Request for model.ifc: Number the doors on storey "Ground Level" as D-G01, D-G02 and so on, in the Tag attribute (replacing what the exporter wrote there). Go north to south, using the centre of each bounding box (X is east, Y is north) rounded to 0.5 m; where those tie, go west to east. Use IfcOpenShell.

First a look at what the model holds.

```python
import ifcopenshell
import ifcopenshell.util.element
import ifcopenshell.util.placement

model = ifcopenshell.open("model.ifc")
print(model.schema)
storey = next(s for s in model.by_type("IfcBuildingStorey") if s.Name == "Ground Level")
doors = [e for e in ifcopenshell.util.element.get_decomposition(storey) if e.is_a("IfcDoor")]
for e in sorted(doors, key=lambda e: e.id()):
    origin = ifcopenshell.util.placement.get_local_placement(e.ObjectPlacement)[:3, 3]
    print(e.id(), e.Tag, e.Name, origin.round(2) + 0.0, sep=" | ")
```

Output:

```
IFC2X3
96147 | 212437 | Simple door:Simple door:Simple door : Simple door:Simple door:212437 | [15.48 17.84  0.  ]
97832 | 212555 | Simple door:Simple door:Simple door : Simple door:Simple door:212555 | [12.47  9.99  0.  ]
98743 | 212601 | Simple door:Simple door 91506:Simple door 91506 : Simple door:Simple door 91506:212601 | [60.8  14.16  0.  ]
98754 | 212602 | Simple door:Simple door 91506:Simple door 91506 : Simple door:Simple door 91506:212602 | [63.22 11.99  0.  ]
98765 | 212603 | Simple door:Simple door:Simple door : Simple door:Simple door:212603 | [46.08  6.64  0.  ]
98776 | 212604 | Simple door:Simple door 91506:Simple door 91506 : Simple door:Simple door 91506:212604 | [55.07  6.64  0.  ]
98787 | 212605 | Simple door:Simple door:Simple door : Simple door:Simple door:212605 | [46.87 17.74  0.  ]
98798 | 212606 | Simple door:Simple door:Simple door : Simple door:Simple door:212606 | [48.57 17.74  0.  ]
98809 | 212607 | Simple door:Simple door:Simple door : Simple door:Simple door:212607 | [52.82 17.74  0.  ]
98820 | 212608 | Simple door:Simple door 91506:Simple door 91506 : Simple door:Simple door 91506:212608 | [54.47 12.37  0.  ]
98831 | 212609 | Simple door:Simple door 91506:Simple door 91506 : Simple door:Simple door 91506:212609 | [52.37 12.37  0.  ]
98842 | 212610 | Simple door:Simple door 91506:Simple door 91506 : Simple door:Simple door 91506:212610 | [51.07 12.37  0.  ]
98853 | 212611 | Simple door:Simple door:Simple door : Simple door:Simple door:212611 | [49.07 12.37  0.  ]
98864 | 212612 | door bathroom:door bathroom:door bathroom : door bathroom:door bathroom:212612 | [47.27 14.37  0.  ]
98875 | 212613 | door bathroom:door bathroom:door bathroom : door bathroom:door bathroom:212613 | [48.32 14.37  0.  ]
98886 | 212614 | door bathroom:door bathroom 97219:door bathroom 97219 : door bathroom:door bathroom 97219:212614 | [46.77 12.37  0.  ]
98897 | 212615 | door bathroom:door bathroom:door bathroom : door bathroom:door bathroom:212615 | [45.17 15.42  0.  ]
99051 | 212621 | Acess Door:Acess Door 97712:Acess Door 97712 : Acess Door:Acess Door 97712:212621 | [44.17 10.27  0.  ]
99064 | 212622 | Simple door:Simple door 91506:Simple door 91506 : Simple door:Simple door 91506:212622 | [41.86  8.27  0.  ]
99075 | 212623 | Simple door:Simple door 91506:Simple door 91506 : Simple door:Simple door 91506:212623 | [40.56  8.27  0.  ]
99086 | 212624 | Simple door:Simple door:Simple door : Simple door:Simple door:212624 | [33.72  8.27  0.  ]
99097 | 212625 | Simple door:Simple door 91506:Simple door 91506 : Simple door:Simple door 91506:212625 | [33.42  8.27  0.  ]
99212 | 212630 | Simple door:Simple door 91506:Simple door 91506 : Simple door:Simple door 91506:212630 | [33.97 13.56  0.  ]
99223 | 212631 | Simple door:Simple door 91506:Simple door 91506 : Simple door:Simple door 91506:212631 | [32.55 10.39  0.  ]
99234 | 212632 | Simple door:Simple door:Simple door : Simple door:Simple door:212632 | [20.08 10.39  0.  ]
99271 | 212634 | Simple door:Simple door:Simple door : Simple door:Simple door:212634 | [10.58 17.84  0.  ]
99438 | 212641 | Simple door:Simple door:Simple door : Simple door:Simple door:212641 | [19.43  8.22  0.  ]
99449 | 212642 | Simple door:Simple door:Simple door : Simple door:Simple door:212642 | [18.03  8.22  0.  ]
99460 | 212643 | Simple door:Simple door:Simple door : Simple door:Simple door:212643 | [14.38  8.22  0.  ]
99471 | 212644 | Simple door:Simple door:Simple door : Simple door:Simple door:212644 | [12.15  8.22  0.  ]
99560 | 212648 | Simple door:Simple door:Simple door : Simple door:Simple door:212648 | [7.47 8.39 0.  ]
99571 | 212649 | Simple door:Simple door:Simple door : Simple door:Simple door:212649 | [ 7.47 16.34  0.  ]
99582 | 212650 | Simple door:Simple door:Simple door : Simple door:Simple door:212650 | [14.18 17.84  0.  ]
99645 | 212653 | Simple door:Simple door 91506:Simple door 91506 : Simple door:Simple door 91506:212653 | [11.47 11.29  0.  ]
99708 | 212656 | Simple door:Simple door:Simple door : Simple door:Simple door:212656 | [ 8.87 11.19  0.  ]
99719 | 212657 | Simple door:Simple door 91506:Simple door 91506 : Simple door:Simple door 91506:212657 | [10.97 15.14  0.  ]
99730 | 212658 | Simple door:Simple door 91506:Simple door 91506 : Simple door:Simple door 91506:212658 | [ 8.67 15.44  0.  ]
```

```python
import ifcopenshell
import ifcopenshell.geom
import ifcopenshell.util.element
import ifcopenshell.util.shape

model = ifcopenshell.open("model.ifc")
settings = ifcopenshell.geom.settings()
settings.set("use-world-coords", True)


def centre(element):
    shape = ifcopenshell.geom.create_shape(settings, element)
    return ifcopenshell.util.shape.get_bbox_centroid(shape.geometry)


storey = next(s for s in model.by_type("IfcBuildingStorey") if s.Name == "Ground Level")
doors = [e for e in ifcopenshell.util.element.get_decomposition(storey) if e.is_a("IfcDoor")]

# Insertion points can sit at a corner or the storey origin, so sort by the geometry (in metres).
centres = {e: centre(e) for e in doors}
doors.sort(key=lambda e: (-round(centres[e][1] / 0.5), centres[e][0]))

for i, e in enumerate(doors, start=1):
    number = f"D-G{i:02d}"
    e.Tag = number
    print(e.id(), number)

model.write("model_edited.ifc")
```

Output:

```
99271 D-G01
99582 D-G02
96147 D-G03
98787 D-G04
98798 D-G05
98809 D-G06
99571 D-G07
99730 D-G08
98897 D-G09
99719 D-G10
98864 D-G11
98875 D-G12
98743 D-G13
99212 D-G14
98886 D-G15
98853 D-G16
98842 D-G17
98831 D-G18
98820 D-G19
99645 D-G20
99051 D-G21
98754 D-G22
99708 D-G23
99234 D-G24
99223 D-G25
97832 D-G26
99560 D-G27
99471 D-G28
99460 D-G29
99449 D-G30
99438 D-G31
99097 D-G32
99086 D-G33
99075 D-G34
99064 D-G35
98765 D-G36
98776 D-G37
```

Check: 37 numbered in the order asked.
